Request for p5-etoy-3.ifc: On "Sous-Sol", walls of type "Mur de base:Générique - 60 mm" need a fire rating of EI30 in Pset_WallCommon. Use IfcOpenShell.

First a look at what the model holds.

```python
import ifcopenshell
import ifcopenshell.util.element

model = ifcopenshell.open("p5-etoy-3.ifc")
print(model.schema)
storey = next(s for s in model.by_type("IfcBuildingStorey") if s.Name == "Sous-Sol")
walls = [e for e in ifcopenshell.util.element.get_decomposition(storey) if e.is_a("IfcWall")]
seen = {}
for e in walls:
    element_type = ifcopenshell.util.element.get_type(e)
    key = (element_type.Name if element_type != e and element_type else None, ifcopenshell.util.element.get_pset(e, "Pset_WallCommon", "FireRating"))
    seen[key] = seen.get(key, 0) + 1
for (name, value), count in sorted(seen.items(), key=str):
    print(count, "x", name, "|", value)
```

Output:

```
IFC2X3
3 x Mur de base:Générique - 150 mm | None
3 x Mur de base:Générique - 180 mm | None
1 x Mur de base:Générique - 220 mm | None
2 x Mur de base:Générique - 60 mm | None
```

```python
import ifcopenshell
import ifcopenshell.api.pset
import ifcopenshell.util.element

model = ifcopenshell.open("p5-etoy-3.ifc")

storey = next(s for s in model.by_type("IfcBuildingStorey") if s.Name == "Sous-Sol")
walls = [e for e in ifcopenshell.util.element.get_decomposition(storey) if e.is_a("IfcWall")]

count = 0
for e in walls:
    element_type = ifcopenshell.util.element.get_type(e)
    if element_type in (None, e) or element_type.Name != "Mur de base:Générique - 60 mm":
        continue
    # add_pset returns the element's existing set when there is one.
    pset = ifcopenshell.api.pset.add_pset(model, product=e, name="Pset_WallCommon")
    ifcopenshell.api.pset.edit_pset(model, pset=pset, properties={"FireRating": "EI30"})
    count += 1

print(count, "walls updated")

model.write("p5-etoy-3-out.ifc")
```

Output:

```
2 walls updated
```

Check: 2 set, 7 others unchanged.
